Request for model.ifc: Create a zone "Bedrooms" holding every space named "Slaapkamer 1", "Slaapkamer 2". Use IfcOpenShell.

First a look at what the model holds.

```python
import ifcopenshell

model = ifcopenshell.open("model.ifc")
print(model.schema)
seen = {}
for space in model.by_type("IfcSpace"):
    seen[space.LongName] = seen.get(space.LongName, 0) + 1
for name, count in sorted(seen.items(), key=str):
    print(count, "x", name)
print("zones:", [z.Name for z in model.by_type("IfcZone")][:20])
```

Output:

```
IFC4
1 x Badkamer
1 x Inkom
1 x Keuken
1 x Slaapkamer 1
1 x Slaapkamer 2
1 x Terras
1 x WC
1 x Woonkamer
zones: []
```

```python
import ifcopenshell
import ifcopenshell.api.group
import ifcopenshell.api.root

model = ifcopenshell.open("model.ifc")

names = {"Slaapkamer 1", "Slaapkamer 2"}
spaces = [s for s in model.by_type("IfcSpace") if s.LongName in names]

zone = ifcopenshell.api.root.create_entity(model, ifc_class="IfcZone", name="Bedrooms")
ifcopenshell.api.group.assign_group(model, products=spaces, group=zone)
print(len(spaces), "spaces in", zone.Name)

model.write("model_v2.ifc")
```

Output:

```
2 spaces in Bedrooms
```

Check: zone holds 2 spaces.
